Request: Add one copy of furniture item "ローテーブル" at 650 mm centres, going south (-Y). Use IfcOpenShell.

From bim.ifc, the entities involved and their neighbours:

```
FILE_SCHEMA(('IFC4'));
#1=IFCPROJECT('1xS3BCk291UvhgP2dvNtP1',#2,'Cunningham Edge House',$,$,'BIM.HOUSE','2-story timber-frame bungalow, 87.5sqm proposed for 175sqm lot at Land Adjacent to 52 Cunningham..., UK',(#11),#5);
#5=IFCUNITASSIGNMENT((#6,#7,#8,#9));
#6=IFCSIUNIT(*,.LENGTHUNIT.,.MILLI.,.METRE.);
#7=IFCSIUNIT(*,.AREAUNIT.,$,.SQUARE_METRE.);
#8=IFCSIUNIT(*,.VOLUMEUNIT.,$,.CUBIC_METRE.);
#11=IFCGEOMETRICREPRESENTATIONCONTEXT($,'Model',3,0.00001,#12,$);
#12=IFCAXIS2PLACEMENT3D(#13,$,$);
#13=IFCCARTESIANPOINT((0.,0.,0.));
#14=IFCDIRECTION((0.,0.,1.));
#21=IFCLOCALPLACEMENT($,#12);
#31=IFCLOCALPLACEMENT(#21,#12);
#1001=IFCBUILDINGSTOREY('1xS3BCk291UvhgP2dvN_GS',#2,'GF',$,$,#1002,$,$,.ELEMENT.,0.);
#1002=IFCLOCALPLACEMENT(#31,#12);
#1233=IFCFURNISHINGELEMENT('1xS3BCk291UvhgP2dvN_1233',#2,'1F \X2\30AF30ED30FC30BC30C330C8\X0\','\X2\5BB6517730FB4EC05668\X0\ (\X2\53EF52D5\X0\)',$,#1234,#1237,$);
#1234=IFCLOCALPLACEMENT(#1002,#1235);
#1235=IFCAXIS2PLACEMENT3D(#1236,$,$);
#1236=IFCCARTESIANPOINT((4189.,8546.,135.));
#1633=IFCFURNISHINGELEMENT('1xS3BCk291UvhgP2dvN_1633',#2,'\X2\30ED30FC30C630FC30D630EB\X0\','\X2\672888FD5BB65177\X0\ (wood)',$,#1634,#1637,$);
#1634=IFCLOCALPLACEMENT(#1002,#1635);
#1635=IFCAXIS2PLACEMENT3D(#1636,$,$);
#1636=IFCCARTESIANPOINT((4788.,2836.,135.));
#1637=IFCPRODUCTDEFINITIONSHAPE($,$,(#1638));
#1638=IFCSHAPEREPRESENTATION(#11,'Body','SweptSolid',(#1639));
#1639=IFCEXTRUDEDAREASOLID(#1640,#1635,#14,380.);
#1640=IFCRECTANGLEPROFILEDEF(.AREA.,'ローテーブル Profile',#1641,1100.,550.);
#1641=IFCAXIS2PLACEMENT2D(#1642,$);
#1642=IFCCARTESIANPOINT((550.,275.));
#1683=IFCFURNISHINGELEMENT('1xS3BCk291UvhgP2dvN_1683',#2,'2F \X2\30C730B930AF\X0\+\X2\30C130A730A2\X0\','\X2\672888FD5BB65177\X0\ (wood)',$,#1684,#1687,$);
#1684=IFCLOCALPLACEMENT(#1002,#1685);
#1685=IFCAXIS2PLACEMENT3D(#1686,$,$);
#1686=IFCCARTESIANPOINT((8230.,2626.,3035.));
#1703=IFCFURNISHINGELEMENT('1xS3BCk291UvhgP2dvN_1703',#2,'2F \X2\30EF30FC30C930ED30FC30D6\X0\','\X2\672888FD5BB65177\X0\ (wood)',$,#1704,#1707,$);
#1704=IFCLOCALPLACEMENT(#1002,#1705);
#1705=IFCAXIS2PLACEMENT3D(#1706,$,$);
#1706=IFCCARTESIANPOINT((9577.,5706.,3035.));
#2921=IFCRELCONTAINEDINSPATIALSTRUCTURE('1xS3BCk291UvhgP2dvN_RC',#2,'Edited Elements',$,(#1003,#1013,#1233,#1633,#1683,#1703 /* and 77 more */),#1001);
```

```python
import numpy as np
import ifcopenshell
import ifcopenshell.api.geometry
import ifcopenshell.api.root
import ifcopenshell.util.element
import ifcopenshell.util.placement

model = ifcopenshell.open("bim.ifc")


def reuse_history(source, copy):
    """copy_class also copies each property set's owner history, people and application; keep the originals."""
    for rel in copy.IsDefinedBy:
        if rel.is_a("IfcRelDefinesByProperties") and (history := rel.RelatingPropertyDefinition.OwnerHistory):
            rel.RelatingPropertyDefinition.OwnerHistory = source.OwnerHistory
            ifcopenshell.util.element.remove_deep2(model, history)


source = model.by_guid("1xS3BCk291UvhgP2dvN_1633")
base = ifcopenshell.util.placement.get_local_placement(source.ObjectPlacement)
step = np.array([0.0, -1.0, 0.0]) * 650.0

for i in range(1, 2):
    copy = ifcopenshell.api.root.copy_class(model, product=source)
    copy.Representation = ifcopenshell.util.element.copy_deep(
        model, source.Representation, exclude=["IfcGeometricRepresentationContext", "IfcRepresentationMap"]
    )
    reuse_history(source, copy)
    matrix = base.copy()
    matrix[:3, 3] += i * step
    print("added at", matrix[:3, 3].round(3) + 0.0)
    ifcopenshell.api.geometry.edit_object_placement(model, product=copy, matrix=matrix, is_si=False)

model.write("bim_v2.ifc")
```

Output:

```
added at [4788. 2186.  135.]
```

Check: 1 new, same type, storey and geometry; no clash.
